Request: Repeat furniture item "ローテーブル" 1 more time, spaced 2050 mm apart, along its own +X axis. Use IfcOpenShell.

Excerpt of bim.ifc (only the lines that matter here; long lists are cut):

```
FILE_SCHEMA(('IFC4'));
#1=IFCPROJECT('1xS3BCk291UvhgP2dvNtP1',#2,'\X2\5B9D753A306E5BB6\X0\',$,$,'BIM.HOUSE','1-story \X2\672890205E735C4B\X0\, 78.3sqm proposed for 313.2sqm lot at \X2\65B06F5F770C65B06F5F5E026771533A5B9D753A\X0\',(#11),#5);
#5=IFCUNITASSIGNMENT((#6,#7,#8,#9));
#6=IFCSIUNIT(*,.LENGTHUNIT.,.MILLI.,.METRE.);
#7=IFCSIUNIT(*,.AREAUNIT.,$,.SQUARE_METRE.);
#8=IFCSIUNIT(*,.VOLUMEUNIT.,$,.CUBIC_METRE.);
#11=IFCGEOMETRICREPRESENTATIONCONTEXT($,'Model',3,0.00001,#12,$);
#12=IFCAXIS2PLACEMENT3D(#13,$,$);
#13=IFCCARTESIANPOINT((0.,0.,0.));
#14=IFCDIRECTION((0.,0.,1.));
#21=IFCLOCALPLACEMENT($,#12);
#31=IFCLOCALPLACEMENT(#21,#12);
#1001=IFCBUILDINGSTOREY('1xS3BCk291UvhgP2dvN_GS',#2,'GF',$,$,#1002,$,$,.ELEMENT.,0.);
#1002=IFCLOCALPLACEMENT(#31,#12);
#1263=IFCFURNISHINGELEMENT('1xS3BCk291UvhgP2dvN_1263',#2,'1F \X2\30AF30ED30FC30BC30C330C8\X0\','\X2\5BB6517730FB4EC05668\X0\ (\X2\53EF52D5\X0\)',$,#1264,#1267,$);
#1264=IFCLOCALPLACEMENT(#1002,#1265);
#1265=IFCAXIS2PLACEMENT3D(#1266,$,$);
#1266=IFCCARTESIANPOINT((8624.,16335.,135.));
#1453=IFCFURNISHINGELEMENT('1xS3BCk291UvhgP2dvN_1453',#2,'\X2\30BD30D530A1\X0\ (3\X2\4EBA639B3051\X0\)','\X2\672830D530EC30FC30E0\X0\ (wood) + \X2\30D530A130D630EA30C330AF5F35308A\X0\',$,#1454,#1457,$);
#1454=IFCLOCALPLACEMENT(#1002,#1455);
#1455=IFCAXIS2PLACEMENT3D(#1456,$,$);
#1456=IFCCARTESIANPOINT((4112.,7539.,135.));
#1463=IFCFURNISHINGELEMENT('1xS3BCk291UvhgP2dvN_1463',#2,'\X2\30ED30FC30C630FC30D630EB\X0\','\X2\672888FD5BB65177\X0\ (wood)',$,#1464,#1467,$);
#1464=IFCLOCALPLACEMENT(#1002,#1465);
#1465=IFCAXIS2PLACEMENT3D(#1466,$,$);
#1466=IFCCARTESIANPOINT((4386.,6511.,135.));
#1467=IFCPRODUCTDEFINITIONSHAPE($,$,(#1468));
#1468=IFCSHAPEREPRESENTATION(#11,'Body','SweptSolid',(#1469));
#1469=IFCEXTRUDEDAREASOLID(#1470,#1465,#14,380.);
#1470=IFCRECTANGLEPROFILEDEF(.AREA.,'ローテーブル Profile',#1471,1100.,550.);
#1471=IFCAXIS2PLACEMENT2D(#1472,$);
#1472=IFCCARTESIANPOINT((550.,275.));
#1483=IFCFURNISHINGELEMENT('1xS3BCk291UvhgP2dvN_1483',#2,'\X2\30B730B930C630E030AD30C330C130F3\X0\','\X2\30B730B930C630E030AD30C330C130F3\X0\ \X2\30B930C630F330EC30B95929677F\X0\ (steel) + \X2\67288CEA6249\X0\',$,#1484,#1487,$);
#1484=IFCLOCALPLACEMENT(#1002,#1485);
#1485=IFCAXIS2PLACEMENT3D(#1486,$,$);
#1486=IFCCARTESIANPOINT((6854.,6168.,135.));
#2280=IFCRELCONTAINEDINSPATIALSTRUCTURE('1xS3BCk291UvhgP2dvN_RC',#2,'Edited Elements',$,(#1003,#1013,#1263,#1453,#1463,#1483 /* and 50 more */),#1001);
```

```python
import ifcopenshell
import ifcopenshell.api.geometry
import ifcopenshell.api.root
import ifcopenshell.util.element
import ifcopenshell.util.placement
import ifcopenshell.util.unit

model = ifcopenshell.open("bim.ifc")
unit_scale = ifcopenshell.util.unit.calculate_unit_scale(model)


def reuse_history(source, copy):
    """copy_class also copies each property set's owner history, people and application; keep the originals."""
    for rel in copy.IsDefinedBy:
        if rel.is_a("IfcRelDefinesByProperties") and (history := rel.RelatingPropertyDefinition.OwnerHistory):
            rel.RelatingPropertyDefinition.OwnerHistory = source.OwnerHistory
            ifcopenshell.util.element.remove_deep2(model, history)


source = model.by_guid("1xS3BCk291UvhgP2dvN_1463")
base = ifcopenshell.util.placement.get_local_placement(source.ObjectPlacement)
step = base[:3, 0] * 2.05 / unit_scale

for i in range(1, 2):
    copy = ifcopenshell.api.root.copy_class(model, product=source)
    copy.Representation = ifcopenshell.util.element.copy_deep(
        model, source.Representation, exclude=["IfcGeometricRepresentationContext", "IfcRepresentationMap"]
    )
    reuse_history(source, copy)
    matrix = base.copy()
    matrix[:3, 3] += i * step
    print("added at", matrix[:3, 3].round(3) + 0.0)
    ifcopenshell.api.geometry.edit_object_placement(model, product=copy, matrix=matrix, is_si=False)

model.write("bim_v2.ifc")
```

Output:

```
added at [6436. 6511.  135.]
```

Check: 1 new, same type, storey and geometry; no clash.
